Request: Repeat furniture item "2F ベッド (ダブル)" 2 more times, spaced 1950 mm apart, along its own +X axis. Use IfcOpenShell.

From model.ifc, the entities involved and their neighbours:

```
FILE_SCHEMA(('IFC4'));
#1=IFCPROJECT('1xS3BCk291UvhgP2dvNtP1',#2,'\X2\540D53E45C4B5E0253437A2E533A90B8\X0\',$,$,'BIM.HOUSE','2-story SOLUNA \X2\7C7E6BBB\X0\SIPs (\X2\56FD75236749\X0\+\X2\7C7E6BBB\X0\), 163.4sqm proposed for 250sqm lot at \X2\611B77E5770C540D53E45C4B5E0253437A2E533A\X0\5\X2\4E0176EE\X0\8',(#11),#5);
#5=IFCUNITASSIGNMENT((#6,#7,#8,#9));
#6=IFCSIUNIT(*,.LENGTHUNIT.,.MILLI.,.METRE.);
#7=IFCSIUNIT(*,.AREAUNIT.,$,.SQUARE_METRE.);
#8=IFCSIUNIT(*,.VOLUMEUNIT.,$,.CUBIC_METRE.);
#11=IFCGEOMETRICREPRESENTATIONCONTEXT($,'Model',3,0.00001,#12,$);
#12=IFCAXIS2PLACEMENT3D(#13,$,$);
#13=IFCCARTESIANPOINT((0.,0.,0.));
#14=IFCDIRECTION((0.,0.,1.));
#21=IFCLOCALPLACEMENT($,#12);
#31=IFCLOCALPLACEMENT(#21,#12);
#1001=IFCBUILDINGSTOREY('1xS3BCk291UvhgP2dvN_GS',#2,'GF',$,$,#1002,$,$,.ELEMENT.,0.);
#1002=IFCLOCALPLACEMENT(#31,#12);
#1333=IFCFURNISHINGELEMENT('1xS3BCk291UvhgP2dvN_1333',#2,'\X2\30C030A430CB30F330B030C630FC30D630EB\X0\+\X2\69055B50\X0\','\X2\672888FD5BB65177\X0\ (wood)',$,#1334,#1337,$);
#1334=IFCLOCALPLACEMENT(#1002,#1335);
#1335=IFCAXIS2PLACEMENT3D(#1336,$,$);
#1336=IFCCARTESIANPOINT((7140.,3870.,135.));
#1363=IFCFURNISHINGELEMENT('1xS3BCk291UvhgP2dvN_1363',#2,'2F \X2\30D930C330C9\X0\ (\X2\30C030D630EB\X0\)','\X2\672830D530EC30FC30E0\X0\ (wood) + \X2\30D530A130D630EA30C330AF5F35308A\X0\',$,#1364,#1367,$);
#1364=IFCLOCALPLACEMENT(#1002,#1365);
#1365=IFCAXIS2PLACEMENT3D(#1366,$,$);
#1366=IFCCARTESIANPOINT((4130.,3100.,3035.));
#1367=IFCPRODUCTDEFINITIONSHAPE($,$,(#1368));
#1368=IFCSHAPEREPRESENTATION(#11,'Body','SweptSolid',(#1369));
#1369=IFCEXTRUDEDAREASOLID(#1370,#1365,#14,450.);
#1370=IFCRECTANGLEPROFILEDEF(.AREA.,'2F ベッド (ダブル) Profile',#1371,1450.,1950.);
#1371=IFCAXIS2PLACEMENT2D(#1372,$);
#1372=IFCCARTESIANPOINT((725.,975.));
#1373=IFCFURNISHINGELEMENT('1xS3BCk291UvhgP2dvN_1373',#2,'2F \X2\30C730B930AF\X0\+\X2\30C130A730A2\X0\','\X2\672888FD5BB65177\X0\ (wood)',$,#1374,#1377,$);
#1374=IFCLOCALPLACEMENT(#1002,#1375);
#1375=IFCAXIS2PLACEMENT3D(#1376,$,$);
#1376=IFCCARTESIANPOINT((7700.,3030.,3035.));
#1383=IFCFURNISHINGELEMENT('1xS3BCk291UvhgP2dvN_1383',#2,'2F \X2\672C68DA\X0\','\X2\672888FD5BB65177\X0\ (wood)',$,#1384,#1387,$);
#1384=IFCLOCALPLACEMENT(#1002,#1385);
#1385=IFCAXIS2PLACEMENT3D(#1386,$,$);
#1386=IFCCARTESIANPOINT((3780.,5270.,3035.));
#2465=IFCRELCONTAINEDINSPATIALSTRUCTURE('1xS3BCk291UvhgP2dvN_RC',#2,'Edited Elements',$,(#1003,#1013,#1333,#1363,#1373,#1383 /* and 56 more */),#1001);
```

```python
import ifcopenshell
import ifcopenshell.api.geometry
import ifcopenshell.api.root
import ifcopenshell.util.element
import ifcopenshell.util.placement
import ifcopenshell.util.unit

model = ifcopenshell.open("model.ifc")
unit_scale = ifcopenshell.util.unit.calculate_unit_scale(model)


def reuse_history(source, copy):
    """copy_class also copies each property set's owner history, people and application; keep the originals."""
    for rel in copy.IsDefinedBy:
        if rel.is_a("IfcRelDefinesByProperties") and (history := rel.RelatingPropertyDefinition.OwnerHistory):
            rel.RelatingPropertyDefinition.OwnerHistory = source.OwnerHistory
            ifcopenshell.util.element.remove_deep2(model, history)


source = model.by_guid("1xS3BCk291UvhgP2dvN_1363")
base = ifcopenshell.util.placement.get_local_placement(source.ObjectPlacement)
step = base[:3, 0] * 1.95 / unit_scale

for i in range(1, 3):
    copy = ifcopenshell.api.root.copy_class(model, product=source)
    copy.Representation = ifcopenshell.util.element.copy_deep(
        model, source.Representation, exclude=["IfcGeometricRepresentationContext", "IfcRepresentationMap"]
    )
    reuse_history(source, copy)
    matrix = base.copy()
    matrix[:3, 3] += i * step
    print("added at", matrix[:3, 3].round(3) + 0.0)
    ifcopenshell.api.geometry.edit_object_placement(model, product=copy, matrix=matrix, is_si=False)

model.write("model_edited.ifc")
```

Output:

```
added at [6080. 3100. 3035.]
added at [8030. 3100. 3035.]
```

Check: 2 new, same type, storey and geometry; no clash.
